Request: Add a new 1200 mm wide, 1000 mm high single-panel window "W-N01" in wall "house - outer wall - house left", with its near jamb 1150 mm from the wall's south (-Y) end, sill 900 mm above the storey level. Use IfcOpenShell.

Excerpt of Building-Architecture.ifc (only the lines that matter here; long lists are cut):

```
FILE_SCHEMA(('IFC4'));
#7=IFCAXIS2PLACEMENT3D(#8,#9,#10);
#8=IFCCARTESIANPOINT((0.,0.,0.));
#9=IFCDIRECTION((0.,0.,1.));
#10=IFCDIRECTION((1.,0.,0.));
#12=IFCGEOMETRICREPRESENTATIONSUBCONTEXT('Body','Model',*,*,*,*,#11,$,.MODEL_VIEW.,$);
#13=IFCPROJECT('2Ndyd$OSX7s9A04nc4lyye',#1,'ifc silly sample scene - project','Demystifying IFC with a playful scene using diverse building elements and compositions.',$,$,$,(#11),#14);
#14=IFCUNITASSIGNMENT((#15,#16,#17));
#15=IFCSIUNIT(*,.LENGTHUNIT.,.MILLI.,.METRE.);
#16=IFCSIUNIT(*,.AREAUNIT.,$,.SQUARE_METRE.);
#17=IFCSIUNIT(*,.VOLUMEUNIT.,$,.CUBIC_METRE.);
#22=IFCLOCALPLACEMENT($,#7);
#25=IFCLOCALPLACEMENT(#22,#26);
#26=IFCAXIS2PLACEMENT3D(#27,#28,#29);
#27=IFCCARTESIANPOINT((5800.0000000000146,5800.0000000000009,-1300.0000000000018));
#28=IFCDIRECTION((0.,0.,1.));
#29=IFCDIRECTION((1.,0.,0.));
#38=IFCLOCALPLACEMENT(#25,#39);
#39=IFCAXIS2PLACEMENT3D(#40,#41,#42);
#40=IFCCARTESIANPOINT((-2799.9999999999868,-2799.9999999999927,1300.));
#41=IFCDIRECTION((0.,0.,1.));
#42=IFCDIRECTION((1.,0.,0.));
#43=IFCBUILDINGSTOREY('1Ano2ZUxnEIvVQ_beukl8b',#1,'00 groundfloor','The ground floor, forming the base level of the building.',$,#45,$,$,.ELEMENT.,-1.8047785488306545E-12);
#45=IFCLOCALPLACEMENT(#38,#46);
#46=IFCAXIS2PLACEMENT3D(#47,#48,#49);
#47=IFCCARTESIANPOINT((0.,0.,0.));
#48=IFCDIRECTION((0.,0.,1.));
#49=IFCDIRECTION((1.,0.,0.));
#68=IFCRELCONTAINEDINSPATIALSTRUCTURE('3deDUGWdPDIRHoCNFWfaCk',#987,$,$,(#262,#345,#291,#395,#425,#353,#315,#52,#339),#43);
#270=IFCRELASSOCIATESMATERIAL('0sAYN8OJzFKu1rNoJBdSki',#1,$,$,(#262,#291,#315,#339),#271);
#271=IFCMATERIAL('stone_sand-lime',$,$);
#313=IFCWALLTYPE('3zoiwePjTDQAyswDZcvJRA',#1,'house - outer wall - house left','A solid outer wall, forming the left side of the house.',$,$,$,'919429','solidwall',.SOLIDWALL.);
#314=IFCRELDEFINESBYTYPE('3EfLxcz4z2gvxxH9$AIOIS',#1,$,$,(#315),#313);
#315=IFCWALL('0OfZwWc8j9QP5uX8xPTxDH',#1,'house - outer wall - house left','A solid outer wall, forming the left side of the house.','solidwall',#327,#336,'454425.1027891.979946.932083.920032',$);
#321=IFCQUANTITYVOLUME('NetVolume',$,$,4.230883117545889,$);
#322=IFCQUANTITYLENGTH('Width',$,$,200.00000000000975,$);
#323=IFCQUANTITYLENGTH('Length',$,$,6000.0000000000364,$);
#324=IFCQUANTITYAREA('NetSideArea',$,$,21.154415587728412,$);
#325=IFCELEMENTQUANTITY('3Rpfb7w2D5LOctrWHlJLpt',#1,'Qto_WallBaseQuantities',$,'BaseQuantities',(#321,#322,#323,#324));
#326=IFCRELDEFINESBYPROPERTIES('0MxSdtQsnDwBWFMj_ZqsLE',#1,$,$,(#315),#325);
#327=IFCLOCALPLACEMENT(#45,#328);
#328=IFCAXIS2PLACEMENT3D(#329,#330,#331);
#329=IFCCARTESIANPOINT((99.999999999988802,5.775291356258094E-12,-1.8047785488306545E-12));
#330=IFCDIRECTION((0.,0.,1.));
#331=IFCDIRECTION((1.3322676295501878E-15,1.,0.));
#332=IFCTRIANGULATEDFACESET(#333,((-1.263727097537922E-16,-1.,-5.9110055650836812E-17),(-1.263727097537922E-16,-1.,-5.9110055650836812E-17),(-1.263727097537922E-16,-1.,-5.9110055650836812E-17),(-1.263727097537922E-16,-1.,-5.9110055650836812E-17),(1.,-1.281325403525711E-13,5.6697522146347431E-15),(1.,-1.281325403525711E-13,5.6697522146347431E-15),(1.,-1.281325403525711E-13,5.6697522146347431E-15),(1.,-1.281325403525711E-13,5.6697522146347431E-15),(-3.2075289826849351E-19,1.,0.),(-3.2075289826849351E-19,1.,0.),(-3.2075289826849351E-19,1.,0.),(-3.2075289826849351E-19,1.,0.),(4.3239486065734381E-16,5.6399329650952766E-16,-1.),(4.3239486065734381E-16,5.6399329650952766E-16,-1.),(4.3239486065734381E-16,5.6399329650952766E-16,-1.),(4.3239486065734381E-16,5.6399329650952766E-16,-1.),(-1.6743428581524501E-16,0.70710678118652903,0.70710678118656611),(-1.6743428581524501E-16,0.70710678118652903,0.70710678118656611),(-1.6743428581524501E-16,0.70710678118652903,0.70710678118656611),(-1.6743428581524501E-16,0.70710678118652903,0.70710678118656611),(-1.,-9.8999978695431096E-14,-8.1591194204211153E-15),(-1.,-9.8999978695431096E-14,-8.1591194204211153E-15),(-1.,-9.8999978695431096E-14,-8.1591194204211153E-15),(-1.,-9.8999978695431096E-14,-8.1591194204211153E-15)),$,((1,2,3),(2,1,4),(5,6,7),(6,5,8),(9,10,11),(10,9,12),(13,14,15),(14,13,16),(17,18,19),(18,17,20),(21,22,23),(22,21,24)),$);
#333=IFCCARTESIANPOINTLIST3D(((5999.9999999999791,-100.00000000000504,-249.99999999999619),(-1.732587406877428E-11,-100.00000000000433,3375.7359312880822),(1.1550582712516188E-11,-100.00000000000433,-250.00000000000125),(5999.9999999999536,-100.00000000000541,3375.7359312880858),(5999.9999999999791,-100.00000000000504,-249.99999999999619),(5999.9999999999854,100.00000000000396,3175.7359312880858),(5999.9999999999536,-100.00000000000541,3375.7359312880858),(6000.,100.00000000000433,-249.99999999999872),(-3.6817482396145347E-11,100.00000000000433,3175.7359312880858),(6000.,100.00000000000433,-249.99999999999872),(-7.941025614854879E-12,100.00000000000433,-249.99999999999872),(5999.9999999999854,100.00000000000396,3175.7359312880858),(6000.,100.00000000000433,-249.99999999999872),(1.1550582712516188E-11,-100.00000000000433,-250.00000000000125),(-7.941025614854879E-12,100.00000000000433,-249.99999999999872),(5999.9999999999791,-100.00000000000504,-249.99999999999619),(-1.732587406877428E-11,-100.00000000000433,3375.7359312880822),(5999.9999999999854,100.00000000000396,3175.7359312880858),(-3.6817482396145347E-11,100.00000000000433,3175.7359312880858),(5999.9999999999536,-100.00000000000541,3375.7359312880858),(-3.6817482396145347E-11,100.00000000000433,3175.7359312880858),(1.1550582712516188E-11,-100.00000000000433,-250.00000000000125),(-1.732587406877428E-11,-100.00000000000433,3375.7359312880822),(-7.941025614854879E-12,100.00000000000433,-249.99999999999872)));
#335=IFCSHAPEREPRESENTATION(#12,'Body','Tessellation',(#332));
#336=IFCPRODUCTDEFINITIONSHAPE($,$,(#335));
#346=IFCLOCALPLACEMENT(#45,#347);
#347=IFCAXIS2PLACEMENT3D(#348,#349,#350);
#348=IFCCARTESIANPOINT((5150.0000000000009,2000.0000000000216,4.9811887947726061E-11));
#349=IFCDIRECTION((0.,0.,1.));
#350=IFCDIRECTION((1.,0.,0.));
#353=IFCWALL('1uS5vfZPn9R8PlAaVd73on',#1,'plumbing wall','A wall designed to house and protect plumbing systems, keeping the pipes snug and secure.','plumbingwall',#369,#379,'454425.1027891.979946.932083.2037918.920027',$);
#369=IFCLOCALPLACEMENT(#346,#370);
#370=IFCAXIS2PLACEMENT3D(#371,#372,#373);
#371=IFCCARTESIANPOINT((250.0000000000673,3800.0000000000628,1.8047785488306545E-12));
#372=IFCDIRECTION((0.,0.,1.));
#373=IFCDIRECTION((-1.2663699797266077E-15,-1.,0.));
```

```python
import numpy as np
import ifcopenshell
import ifcopenshell.api.feature
import ifcopenshell.api.geometry
import ifcopenshell.api.pset
import ifcopenshell.api.root
import ifcopenshell.api.spatial
import ifcopenshell.geom
import ifcopenshell.util.element
import ifcopenshell.util.placement
import ifcopenshell.util.representation
import ifcopenshell.util.shape
import ifcopenshell.util.unit

model = ifcopenshell.open("Building-Architecture.ifc")
unit_scale = ifcopenshell.util.unit.calculate_unit_scale(model)
area_scale = ifcopenshell.util.unit.calculate_unit_scale(model, "AREAUNIT")
volume_scale = ifcopenshell.util.unit.calculate_unit_scale(model, "VOLUMEUNIT")
settings = ifcopenshell.geom.settings()


def volume(element):
    """Net volume in cubic metres, openings subtracted."""
    shape = ifcopenshell.geom.create_shape(settings, element)
    return ifcopenshell.util.shape.get_volume(shape.geometry)


wall = model.by_guid("0OfZwWc8j9QP5uX8xPTxDH")
storey = ifcopenshell.util.element.get_container(wall, ifc_class="IfcBuildingStorey")
context = ifcopenshell.util.representation.get_context(model, "Model", "Body", "MODEL_VIEW")
before = volume(wall)

width, height, from_end, sill = 1.2, 1, 1.15, 0.9  # metres

# The wall runs along its own X axis, and the end named is its -X end.
wall_shape = ifcopenshell.geom.create_shape(settings, wall)
x, y, z = ifcopenshell.util.shape.get_vertices(wall_shape.geometry).T
start = x.min() + from_end
face, thickness = float(y.min()), float(y.max() - y.min())
wall_matrix = ifcopenshell.util.placement.get_local_placement(wall.ObjectPlacement)
level = ifcopenshell.util.placement.get_local_placement(storey.ObjectPlacement)[2, 3]


def in_wall(x, y):
    """Placement at x, y metres in the wall's axes, at sill height."""
    matrix = wall_matrix.copy()
    matrix[:, 3] = wall_matrix @ np.array([x / unit_scale, y / unit_scale, 0.0, 1.0])
    matrix[2, 3] = level + sill / unit_scale
    return matrix


# Opening: a box that overshoots both wall faces by 50 mm.
opening = ifcopenshell.api.root.create_entity(model, ifc_class="IfcOpeningElement", predefined_type="OPENING")
box = ifcopenshell.api.geometry.add_wall_representation(
    model, context=context, length=width, height=height, thickness=thickness + 0.1
)
ifcopenshell.api.geometry.assign_representation(model, product=opening, representation=box)
ifcopenshell.api.geometry.edit_object_placement(model, product=opening, matrix=in_wall(start, face - 0.05), is_si=False)
ifcopenshell.api.feature.add_feature(model, feature=opening, element=wall)

window = ifcopenshell.api.root.create_entity(model, ifc_class="IfcWindow", name="W-N01", predefined_type="WINDOW")
window.OverallWidth, window.OverallHeight = width / unit_scale, height / unit_scale
window.PartitioningType = "SINGLE_PANEL"
body = ifcopenshell.api.geometry.add_window_representation(
    model,
    context=context,
    overall_width=window.OverallWidth,
    overall_height=window.OverallHeight,
    partition_type="SINGLE_PANEL",
)
ifcopenshell.api.geometry.assign_representation(model, product=window, representation=body)
ifcopenshell.api.spatial.assign_container(model, products=[window], relating_structure=storey)
ifcopenshell.api.feature.add_filling(model, opening=opening, element=window)

# Centre the window in the wall's thickness.
ifcopenshell.api.geometry.edit_object_placement(model, product=window, matrix=in_wall(start, face), is_si=False)
window_shape = ifcopenshell.geom.create_shape(settings, window)
depth = ifcopenshell.util.shape.get_vertices(window_shape.geometry)[:, 1]
offset = face + thickness / 2 - (depth.min() + depth.max()) / 2
ifcopenshell.api.geometry.edit_object_placement(model, product=window, matrix=in_wall(start, offset), is_si=False)

after = volume(wall)

# Update the wall's stored quantities.
qto = model.by_id(ifcopenshell.util.element.get_pset(wall, "Qto_WallBaseQuantities", should_inherit=False)["id"])
ifcopenshell.api.pset.edit_qto(model, qto=qto, properties={
    "NetVolume": after / volume_scale,
    "NetSideArea": after / thickness / area_scale,
})

print(f"wall volume {before:.3f} -> {after:.3f} m3")

model.write("Building-Architecture-out.ifc")
```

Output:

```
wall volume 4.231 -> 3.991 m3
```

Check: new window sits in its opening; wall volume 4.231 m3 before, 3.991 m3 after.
